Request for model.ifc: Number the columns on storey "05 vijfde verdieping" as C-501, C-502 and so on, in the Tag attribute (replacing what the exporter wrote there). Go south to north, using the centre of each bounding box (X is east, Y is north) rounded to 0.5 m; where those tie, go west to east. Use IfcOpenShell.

First a look at what the model holds.

```python
import ifcopenshell
import ifcopenshell.util.element
import ifcopenshell.util.placement

model = ifcopenshell.open("model.ifc")
print(model.schema)
storey = next(s for s in model.by_type("IfcBuildingStorey") if s.Name == "05 vijfde verdieping")
columns = [e for e in ifcopenshell.util.element.get_decomposition(storey) if e.is_a("IfcColumn")]
for e in sorted(columns, key=lambda e: e.id()):
    origin = ifcopenshell.util.placement.get_local_placement(e.ObjectPlacement)[:3, 3]
    print(e.id(), e.Tag, e.Name, origin.round(2) + 0.0, sep=" | ")
```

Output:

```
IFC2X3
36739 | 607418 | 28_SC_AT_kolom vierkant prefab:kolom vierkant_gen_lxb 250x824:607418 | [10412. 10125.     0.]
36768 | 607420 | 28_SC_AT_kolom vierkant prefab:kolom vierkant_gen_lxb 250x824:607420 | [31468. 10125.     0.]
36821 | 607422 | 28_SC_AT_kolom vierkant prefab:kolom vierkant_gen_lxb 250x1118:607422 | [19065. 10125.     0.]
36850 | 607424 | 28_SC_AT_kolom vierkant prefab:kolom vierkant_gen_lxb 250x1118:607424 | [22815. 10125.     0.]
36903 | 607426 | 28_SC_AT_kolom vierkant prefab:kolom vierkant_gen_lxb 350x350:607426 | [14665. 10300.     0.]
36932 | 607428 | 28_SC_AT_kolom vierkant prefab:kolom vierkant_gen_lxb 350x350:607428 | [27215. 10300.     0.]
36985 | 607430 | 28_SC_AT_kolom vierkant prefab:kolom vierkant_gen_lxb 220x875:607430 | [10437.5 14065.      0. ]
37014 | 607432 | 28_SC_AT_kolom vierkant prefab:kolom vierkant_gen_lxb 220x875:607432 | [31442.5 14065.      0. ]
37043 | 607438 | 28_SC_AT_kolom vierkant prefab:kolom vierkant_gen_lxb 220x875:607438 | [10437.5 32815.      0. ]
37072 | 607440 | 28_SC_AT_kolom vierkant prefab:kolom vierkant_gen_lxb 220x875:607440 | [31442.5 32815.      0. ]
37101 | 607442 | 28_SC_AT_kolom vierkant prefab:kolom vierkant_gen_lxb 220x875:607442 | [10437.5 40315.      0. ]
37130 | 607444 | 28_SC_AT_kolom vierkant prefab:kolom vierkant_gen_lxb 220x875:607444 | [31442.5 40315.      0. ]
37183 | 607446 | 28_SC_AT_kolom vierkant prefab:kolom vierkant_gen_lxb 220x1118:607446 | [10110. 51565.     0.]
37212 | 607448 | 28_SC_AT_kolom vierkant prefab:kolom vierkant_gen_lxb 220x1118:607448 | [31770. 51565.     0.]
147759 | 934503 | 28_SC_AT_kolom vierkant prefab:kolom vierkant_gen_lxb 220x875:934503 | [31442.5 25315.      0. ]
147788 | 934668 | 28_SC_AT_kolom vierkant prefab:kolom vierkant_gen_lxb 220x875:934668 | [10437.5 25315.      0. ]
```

```python
import ifcopenshell
import ifcopenshell.geom
import ifcopenshell.util.element
import ifcopenshell.util.shape

model = ifcopenshell.open("model.ifc")
settings = ifcopenshell.geom.settings()
settings.set("use-world-coords", True)


def centre(element):
    shape = ifcopenshell.geom.create_shape(settings, element)
    return ifcopenshell.util.shape.get_bbox_centroid(shape.geometry)


storey = next(s for s in model.by_type("IfcBuildingStorey") if s.Name == "05 vijfde verdieping")
columns = [e for e in ifcopenshell.util.element.get_decomposition(storey) if e.is_a("IfcColumn")]

# Insertion points can sit at a corner or the storey origin, so sort by the geometry (in metres).
centres = {e: centre(e) for e in columns}
columns.sort(key=lambda e: (round(centres[e][1] / 0.5), centres[e][0]))

for i, e in enumerate(columns, start=1):
    number = f"C-5{i:02d}"
    e.Tag = number
    print(e.id(), number)

model.write("model_updated.ifc")
```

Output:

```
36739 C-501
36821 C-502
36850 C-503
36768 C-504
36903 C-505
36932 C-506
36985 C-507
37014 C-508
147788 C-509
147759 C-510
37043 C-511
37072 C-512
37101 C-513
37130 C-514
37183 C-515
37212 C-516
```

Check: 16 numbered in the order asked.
